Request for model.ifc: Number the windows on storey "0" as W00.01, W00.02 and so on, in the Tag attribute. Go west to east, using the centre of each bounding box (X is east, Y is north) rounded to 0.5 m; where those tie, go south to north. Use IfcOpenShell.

First a look at what the model holds.

```python
import ifcopenshell
import ifcopenshell.util.element
import ifcopenshell.util.placement

model = ifcopenshell.open("model.ifc")
print(model.schema)
storey = next(s for s in model.by_type("IfcBuildingStorey") if s.Name == "0")
windows = [e for e in ifcopenshell.util.element.get_decomposition(storey) if e.is_a("IfcWindow")]
for e in sorted(windows, key=lambda e: e.id()):
    origin = ifcopenshell.util.placement.get_local_placement(e.ObjectPlacement)[:3, 3]
    print(e.id(), e.Tag, e.Name, origin.round(2) + 0.0, sep=" | ")
```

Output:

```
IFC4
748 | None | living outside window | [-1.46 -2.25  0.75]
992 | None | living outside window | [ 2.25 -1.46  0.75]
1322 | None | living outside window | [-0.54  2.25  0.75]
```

```python
import ifcopenshell
import ifcopenshell.geom
import ifcopenshell.util.element
import ifcopenshell.util.shape

model = ifcopenshell.open("model.ifc")
settings = ifcopenshell.geom.settings()
settings.set("use-world-coords", True)


def centre(element):
    shape = ifcopenshell.geom.create_shape(settings, element)
    return ifcopenshell.util.shape.get_bbox_centroid(shape.geometry)


storey = next(s for s in model.by_type("IfcBuildingStorey") if s.Name == "0")
windows = [e for e in ifcopenshell.util.element.get_decomposition(storey) if e.is_a("IfcWindow")]

# Insertion points can sit at a corner or the storey origin, so sort by the geometry (in metres).
centres = {e: centre(e) for e in windows}
windows.sort(key=lambda e: (round(centres[e][0] / 0.5), centres[e][1]))

for i, e in enumerate(windows, start=1):
    number = f"W00.{i:02d}"
    e.Tag = number
    print(e.id(), number)

model.write("model_rev.ifc")
```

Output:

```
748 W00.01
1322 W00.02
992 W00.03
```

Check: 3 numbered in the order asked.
